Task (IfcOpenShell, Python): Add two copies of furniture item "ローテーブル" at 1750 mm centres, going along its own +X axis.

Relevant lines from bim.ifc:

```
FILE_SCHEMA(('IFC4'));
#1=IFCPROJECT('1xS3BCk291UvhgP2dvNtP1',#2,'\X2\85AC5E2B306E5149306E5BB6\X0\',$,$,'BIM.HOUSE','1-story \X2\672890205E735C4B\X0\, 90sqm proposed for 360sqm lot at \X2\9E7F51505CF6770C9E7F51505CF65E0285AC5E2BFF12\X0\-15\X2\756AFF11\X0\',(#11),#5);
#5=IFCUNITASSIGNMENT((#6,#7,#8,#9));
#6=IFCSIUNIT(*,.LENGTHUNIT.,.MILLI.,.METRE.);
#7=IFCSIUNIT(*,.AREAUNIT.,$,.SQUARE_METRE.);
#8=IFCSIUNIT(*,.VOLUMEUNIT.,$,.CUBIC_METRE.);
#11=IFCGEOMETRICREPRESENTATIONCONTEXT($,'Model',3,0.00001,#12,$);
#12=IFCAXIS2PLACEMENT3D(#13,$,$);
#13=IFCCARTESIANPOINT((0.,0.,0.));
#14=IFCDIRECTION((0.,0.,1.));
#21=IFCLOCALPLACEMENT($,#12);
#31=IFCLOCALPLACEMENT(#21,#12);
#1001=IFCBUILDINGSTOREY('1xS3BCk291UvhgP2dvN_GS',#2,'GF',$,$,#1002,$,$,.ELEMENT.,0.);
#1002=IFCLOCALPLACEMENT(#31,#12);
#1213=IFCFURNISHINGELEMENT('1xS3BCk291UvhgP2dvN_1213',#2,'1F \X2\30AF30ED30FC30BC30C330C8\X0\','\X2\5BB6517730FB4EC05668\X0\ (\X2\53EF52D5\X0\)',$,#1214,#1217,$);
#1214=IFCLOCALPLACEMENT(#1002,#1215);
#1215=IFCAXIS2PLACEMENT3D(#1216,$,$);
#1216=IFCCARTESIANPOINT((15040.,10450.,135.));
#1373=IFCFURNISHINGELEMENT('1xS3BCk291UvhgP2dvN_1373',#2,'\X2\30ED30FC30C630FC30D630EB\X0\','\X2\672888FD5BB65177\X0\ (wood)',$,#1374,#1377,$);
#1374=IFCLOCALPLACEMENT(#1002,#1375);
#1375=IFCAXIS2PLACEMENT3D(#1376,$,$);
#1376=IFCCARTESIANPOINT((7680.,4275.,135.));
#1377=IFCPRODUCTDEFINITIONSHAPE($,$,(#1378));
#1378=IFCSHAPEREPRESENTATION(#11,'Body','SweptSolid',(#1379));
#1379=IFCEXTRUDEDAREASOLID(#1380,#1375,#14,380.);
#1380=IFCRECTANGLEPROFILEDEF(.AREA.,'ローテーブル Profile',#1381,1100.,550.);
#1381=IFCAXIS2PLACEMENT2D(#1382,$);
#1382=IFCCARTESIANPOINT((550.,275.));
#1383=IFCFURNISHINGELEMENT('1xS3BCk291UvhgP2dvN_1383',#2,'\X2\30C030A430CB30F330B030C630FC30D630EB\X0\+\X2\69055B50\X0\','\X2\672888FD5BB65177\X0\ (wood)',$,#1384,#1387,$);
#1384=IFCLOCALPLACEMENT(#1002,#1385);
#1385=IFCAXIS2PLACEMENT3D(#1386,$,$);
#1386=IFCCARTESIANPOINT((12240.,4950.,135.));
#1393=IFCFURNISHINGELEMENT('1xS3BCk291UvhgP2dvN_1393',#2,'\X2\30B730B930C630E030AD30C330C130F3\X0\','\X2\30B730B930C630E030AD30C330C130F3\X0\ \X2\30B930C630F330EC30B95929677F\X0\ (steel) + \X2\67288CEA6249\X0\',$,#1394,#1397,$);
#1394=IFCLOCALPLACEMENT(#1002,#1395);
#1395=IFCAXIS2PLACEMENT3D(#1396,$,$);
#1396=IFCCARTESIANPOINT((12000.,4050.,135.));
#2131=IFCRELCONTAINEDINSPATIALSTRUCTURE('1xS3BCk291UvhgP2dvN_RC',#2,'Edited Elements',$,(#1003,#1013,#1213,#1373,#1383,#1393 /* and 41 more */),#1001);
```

```python
import ifcopenshell
import ifcopenshell.api.geometry
import ifcopenshell.api.root
import ifcopenshell.util.element
import ifcopenshell.util.placement
import ifcopenshell.util.unit

model = ifcopenshell.open("bim.ifc")
unit_scale = ifcopenshell.util.unit.calculate_unit_scale(model)


def reuse_history(source, copy):
    """copy_class also copies each property set's owner history, people and application; keep the originals."""
    for rel in copy.IsDefinedBy:
        if rel.is_a("IfcRelDefinesByProperties") and (history := rel.RelatingPropertyDefinition.OwnerHistory):
            rel.RelatingPropertyDefinition.OwnerHistory = source.OwnerHistory
            ifcopenshell.util.element.remove_deep2(model, history)


source = model.by_id(1373)
base = ifcopenshell.util.placement.get_local_placement(source.ObjectPlacement)
step = base[:3, 0] * 1.75 / unit_scale

for i in range(1, 3):
    copy = ifcopenshell.api.root.copy_class(model, product=source)
    copy.Representation = ifcopenshell.util.element.copy_deep(
        model, source.Representation, exclude=["IfcGeometricRepresentationContext", "IfcRepresentationMap"]
    )
    reuse_history(source, copy)
    matrix = base.copy()
    matrix[:3, 3] += i * step
    print("added at", matrix[:3, 3].round(3) + 0.0)
    ifcopenshell.api.geometry.edit_object_placement(model, product=copy, matrix=matrix, is_si=False)

model.write("bim_rev.ifc")
```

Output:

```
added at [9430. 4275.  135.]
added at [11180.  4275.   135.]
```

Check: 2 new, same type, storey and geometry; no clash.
